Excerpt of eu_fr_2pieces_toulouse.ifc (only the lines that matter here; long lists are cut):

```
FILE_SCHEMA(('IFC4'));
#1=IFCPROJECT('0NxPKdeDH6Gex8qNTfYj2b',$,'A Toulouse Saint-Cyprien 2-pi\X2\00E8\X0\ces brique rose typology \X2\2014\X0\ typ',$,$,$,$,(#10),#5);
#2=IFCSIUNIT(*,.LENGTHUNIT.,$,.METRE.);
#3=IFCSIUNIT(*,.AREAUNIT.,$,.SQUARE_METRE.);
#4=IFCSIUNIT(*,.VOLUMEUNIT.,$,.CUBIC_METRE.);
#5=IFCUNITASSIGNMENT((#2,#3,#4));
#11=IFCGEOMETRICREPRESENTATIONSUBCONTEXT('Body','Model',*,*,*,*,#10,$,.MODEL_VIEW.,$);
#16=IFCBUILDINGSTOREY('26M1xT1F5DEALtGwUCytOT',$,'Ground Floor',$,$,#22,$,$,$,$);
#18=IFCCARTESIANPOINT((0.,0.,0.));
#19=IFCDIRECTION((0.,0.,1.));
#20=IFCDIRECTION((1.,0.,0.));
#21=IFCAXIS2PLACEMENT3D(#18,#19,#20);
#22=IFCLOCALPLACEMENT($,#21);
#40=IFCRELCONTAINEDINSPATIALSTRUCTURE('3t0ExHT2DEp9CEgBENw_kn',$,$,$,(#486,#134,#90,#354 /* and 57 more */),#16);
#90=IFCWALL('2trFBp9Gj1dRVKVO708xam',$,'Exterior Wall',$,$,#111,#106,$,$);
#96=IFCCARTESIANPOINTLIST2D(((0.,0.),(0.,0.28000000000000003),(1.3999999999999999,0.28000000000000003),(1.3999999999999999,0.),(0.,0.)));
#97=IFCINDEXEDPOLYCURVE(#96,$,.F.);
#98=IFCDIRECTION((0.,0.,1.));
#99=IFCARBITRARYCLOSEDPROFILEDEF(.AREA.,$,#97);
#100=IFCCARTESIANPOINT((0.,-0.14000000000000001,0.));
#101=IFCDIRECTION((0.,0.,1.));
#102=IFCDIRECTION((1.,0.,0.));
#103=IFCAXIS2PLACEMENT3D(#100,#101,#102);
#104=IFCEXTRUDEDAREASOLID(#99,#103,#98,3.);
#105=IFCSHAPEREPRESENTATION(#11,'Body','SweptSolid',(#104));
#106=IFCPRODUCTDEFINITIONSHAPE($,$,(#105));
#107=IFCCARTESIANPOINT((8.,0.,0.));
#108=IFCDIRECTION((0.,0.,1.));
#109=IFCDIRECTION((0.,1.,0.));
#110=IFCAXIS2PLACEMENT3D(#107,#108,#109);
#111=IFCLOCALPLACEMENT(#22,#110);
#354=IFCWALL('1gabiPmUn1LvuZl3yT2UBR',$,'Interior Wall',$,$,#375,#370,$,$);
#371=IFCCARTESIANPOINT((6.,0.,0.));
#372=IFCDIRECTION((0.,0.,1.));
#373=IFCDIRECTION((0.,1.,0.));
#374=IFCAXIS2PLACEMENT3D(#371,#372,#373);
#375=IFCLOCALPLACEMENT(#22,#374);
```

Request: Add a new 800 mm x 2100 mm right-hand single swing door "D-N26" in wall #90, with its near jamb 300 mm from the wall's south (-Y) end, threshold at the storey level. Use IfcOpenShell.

```python
import numpy as np
import ifcopenshell
import ifcopenshell.api.feature
import ifcopenshell.api.geometry
import ifcopenshell.api.root
import ifcopenshell.api.spatial
import ifcopenshell.geom
import ifcopenshell.util.element
import ifcopenshell.util.placement
import ifcopenshell.util.representation
import ifcopenshell.util.shape
import ifcopenshell.util.unit

model = ifcopenshell.open("eu_fr_2pieces_toulouse.ifc")
unit_scale = ifcopenshell.util.unit.calculate_unit_scale(model)
settings = ifcopenshell.geom.settings()


def volume(element):
    """Net volume in cubic metres, openings subtracted."""
    shape = ifcopenshell.geom.create_shape(settings, element)
    return ifcopenshell.util.shape.get_volume(shape.geometry)


wall = model.by_guid("2trFBp9Gj1dRVKVO708xam")
storey = ifcopenshell.util.element.get_container(wall, ifc_class="IfcBuildingStorey")
context = ifcopenshell.util.representation.get_context(model, "Model", "Body", "MODEL_VIEW")
before = volume(wall)

width, height, from_end, sill = 0.8, 2.1, 0.3, 0.0  # metres

# The wall runs along its own X axis, and the end named is its -X end.
wall_shape = ifcopenshell.geom.create_shape(settings, wall)
x, y, z = ifcopenshell.util.shape.get_vertices(wall_shape.geometry).T
start = x.min() + from_end
face, thickness = float(y.min()), float(y.max() - y.min())
wall_matrix = ifcopenshell.util.placement.get_local_placement(wall.ObjectPlacement)
level = ifcopenshell.util.placement.get_local_placement(storey.ObjectPlacement)[2, 3]


def in_wall(x, y):
    """Placement at x, y metres in the wall's axes, at sill height."""
    matrix = wall_matrix.copy()
    matrix[:, 3] = wall_matrix @ np.array([x / unit_scale, y / unit_scale, 0.0, 1.0])
    matrix[2, 3] = level + sill / unit_scale
    return matrix


# Opening: a box that overshoots both wall faces by 50 mm.
opening = ifcopenshell.api.root.create_entity(model, ifc_class="IfcOpeningElement", predefined_type="OPENING")
box = ifcopenshell.api.geometry.add_wall_representation(
    model, context=context, length=width, height=height, thickness=thickness + 0.1
)
ifcopenshell.api.geometry.assign_representation(model, product=opening, representation=box)
ifcopenshell.api.geometry.edit_object_placement(model, product=opening, matrix=in_wall(start, face - 0.05), is_si=False)
ifcopenshell.api.feature.add_feature(model, feature=opening, element=wall)

door = ifcopenshell.api.root.create_entity(model, ifc_class="IfcDoor", name="D-N26", predefined_type="DOOR")
door.OverallWidth, door.OverallHeight = width / unit_scale, height / unit_scale
door.OperationType = "SINGLE_SWING_RIGHT"
body = ifcopenshell.api.geometry.add_door_representation(
    model,
    context=context,
    overall_width=door.OverallWidth,
    overall_height=door.OverallHeight,
    operation_type="SINGLE_SWING_RIGHT",
    lining_properties={"LiningDepth": thickness / unit_scale, "ThresholdDepth": thickness / unit_scale},
)
ifcopenshell.api.geometry.assign_representation(model, product=door, representation=body)
ifcopenshell.api.spatial.assign_container(model, products=[door], relating_structure=storey)
ifcopenshell.api.feature.add_filling(model, opening=opening, element=door)

# The lining spans the wall, so the door starts at the wall face.
ifcopenshell.api.geometry.edit_object_placement(model, product=door, matrix=in_wall(start, face), is_si=False)

after = volume(wall)

print(f"wall volume {before:.3f} -> {after:.3f} m3")

model.write("eu_fr_2pieces_toulouse_rev.ifc")
```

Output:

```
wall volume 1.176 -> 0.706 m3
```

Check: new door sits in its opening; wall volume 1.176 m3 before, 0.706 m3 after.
